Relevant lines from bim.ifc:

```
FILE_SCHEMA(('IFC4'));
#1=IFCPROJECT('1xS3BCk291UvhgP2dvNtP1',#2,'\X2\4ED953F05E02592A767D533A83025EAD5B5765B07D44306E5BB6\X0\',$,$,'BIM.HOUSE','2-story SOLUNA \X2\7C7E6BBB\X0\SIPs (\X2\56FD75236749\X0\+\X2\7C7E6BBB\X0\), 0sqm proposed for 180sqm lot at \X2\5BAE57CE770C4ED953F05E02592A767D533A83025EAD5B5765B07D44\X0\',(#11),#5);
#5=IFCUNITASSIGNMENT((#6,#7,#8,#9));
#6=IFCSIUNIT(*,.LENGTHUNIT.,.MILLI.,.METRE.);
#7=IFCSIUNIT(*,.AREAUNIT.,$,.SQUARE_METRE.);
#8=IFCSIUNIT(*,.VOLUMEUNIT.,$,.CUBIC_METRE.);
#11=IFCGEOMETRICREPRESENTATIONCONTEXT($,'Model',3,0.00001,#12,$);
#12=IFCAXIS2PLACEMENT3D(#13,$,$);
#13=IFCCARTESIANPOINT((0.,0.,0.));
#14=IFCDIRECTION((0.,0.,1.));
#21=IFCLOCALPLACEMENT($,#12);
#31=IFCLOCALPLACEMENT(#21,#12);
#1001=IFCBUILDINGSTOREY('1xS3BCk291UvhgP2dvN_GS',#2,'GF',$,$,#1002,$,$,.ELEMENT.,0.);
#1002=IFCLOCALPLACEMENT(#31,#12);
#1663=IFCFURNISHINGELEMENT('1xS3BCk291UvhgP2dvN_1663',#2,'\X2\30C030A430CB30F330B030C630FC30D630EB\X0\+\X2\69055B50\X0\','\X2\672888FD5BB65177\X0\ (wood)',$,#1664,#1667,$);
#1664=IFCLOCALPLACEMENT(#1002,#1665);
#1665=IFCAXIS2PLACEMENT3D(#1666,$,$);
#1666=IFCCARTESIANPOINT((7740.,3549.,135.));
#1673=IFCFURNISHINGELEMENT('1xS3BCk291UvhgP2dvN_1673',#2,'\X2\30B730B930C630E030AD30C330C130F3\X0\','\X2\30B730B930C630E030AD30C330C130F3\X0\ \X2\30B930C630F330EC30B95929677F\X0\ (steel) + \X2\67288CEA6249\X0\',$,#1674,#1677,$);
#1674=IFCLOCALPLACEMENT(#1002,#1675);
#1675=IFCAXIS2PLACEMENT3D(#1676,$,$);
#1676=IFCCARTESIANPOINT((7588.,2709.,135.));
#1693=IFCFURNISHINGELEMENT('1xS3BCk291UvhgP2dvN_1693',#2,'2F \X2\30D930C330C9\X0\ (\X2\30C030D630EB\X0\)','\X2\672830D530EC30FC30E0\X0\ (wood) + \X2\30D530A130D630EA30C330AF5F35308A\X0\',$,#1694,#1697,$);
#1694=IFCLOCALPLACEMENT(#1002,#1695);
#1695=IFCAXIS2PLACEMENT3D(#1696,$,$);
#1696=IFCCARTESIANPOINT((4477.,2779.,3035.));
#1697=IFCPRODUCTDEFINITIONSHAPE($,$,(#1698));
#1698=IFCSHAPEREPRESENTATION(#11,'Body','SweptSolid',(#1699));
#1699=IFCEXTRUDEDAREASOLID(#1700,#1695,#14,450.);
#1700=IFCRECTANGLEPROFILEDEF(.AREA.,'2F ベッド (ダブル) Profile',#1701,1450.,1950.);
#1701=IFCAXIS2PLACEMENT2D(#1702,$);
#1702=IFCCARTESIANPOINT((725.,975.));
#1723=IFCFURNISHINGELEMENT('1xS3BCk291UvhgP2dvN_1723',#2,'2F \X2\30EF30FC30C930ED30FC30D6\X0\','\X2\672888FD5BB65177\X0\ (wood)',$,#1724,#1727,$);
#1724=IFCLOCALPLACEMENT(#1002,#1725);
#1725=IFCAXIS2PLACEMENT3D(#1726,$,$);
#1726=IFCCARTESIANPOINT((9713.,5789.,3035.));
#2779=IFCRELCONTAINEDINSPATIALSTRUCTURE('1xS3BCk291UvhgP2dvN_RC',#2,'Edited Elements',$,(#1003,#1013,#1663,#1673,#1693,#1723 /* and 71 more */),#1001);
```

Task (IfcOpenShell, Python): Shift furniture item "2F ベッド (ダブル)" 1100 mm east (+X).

```python
import ifcopenshell
import ifcopenshell.api.geometry
import ifcopenshell.util.placement
import ifcopenshell.util.unit

model = ifcopenshell.open("bim.ifc")
unit_scale = ifcopenshell.util.unit.calculate_unit_scale(model)

item = model.by_guid("1xS3BCk291UvhgP2dvN_1693")
matrix = ifcopenshell.util.placement.get_local_placement(item.ObjectPlacement)
matrix[0, 3] += 1.1 / unit_scale
ifcopenshell.api.geometry.edit_object_placement(model, product=item, matrix=matrix, is_si=False)

print(ifcopenshell.util.placement.get_local_placement(item.ObjectPlacement).round(3) + 0.0)

model.write("bim_v2.ifc")
```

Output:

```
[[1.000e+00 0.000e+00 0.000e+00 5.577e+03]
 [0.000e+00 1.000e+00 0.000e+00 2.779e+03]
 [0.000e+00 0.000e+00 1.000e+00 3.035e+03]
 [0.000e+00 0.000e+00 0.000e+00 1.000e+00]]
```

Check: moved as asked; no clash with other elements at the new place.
